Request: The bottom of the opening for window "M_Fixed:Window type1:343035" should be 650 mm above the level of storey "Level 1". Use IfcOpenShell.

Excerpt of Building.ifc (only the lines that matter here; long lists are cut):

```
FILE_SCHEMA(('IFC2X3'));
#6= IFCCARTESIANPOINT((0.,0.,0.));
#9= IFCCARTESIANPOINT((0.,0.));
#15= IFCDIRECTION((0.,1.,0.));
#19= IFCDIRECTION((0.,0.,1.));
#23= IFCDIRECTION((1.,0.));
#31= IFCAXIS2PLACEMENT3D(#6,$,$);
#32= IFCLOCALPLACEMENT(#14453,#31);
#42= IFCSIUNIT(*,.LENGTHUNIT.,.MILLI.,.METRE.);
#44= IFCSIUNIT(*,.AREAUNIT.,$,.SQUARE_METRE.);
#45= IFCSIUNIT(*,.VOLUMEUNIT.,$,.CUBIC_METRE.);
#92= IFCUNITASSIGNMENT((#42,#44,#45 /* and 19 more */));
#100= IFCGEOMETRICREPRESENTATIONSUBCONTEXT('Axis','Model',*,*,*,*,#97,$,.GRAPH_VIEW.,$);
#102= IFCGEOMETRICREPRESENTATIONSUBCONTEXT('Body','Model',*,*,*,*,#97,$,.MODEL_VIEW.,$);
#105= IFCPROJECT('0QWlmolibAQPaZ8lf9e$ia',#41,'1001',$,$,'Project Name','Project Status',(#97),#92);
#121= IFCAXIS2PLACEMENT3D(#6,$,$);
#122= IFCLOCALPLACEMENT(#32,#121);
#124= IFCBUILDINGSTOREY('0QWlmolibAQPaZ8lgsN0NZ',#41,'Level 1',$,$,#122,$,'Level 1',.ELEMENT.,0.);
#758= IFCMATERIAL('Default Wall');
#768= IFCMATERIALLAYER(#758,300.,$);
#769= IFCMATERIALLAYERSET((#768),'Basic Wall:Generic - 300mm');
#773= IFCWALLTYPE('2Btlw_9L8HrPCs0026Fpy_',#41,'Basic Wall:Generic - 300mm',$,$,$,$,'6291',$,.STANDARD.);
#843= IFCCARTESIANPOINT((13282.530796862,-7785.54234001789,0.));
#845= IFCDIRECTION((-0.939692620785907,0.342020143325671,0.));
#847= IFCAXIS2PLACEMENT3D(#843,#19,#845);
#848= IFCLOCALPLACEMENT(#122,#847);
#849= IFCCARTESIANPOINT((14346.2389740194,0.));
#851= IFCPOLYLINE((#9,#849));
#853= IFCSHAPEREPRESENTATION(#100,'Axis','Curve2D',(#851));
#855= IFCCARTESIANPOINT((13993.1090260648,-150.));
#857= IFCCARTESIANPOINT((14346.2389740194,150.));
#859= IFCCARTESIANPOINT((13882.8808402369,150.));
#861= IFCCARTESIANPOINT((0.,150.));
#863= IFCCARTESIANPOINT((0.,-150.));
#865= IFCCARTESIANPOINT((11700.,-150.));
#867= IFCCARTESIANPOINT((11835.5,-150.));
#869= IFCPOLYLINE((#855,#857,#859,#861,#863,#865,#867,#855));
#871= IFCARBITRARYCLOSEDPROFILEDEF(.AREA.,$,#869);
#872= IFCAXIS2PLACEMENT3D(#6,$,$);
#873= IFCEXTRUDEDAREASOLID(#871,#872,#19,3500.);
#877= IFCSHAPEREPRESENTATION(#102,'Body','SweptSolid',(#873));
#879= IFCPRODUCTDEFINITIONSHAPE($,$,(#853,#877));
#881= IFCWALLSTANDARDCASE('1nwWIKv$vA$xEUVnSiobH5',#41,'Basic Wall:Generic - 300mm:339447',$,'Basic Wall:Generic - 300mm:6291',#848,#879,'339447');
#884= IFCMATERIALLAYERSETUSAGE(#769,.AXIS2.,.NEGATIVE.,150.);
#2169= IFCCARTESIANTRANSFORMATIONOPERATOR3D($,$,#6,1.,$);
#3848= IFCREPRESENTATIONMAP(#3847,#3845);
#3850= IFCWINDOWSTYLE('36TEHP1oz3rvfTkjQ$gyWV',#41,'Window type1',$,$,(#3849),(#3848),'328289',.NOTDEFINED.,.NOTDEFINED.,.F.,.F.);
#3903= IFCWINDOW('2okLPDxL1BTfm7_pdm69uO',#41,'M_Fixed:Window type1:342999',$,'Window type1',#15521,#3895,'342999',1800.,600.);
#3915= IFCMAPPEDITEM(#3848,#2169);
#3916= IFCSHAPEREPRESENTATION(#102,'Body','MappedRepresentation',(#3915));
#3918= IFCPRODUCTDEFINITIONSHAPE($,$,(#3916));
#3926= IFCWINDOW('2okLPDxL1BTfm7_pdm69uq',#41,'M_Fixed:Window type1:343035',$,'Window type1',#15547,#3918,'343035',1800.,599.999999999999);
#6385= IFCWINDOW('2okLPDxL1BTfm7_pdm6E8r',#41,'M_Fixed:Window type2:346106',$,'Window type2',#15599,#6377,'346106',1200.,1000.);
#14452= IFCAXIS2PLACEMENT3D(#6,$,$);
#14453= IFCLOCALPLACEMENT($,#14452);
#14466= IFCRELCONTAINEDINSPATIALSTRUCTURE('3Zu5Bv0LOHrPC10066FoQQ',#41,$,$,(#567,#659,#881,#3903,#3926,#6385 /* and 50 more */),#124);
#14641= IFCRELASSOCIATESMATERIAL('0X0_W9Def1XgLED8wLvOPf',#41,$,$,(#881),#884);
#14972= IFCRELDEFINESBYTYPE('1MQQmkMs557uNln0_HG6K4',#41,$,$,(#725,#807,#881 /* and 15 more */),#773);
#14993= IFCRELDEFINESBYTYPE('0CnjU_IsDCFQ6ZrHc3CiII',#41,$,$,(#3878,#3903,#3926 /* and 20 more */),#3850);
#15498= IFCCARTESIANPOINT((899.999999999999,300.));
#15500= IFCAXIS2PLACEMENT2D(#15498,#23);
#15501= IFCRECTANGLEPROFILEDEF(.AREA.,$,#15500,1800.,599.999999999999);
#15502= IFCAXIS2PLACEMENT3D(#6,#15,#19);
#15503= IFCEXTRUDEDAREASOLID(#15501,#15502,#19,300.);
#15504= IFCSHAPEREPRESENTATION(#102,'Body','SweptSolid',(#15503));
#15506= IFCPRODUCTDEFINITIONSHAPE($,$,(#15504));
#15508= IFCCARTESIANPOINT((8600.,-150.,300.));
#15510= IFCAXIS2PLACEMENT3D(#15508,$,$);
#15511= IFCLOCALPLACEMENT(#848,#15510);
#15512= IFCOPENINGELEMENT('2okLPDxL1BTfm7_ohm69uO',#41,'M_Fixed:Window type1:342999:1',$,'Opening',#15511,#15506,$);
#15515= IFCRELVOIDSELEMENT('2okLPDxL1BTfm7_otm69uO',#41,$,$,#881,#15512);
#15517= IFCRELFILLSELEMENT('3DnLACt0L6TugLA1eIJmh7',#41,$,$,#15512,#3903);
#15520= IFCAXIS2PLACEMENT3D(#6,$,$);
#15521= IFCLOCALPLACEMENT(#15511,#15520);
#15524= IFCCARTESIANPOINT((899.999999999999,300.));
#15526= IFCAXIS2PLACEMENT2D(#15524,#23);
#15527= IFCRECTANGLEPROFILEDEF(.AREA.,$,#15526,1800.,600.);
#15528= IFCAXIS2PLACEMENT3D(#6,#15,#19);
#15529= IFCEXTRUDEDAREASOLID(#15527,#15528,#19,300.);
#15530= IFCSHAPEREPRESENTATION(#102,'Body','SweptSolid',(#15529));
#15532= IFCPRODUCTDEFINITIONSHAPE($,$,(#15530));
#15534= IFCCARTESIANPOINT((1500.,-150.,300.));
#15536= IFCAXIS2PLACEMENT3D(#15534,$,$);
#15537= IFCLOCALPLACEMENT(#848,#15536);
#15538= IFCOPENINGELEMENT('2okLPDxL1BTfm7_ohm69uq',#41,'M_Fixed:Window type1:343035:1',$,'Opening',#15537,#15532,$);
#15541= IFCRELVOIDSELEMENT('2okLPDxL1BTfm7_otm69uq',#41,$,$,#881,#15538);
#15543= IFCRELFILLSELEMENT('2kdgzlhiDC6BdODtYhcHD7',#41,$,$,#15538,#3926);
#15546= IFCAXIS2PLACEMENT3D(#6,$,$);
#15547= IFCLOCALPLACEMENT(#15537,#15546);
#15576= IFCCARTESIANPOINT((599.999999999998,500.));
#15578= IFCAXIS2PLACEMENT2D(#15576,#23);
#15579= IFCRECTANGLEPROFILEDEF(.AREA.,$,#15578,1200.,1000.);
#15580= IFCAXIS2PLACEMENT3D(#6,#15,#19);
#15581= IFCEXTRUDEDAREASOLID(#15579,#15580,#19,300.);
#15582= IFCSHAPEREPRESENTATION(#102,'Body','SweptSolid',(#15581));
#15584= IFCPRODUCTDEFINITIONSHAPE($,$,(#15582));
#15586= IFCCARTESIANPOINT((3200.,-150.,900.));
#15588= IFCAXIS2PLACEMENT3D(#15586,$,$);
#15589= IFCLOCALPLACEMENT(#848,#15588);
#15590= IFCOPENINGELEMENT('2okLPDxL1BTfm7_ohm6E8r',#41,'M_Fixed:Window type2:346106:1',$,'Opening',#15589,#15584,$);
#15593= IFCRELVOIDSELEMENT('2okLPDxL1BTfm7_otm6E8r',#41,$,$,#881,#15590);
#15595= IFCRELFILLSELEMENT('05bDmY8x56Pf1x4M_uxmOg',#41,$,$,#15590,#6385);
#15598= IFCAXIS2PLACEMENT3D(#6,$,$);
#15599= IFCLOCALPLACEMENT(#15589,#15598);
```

```python
import numpy as np
import ifcopenshell
import ifcopenshell.api.geometry
import ifcopenshell.geom
import ifcopenshell.util.element
import ifcopenshell.util.placement
import ifcopenshell.util.shape
import ifcopenshell.util.unit

model = ifcopenshell.open("Building.ifc")
unit_scale = ifcopenshell.util.unit.calculate_unit_scale(model)

window = model.by_guid("2okLPDxL1BTfm7_pdm69uq")
opening = window.FillsVoids[0].RelatingOpeningElement
storey = ifcopenshell.util.element.get_container(window, ifc_class="IfcBuildingStorey")
level = ifcopenshell.util.placement.get_local_placement(storey.ObjectPlacement)[2, 3]

# The opening's origin need not be at the sill, so measure its lowest point.
shape = ifcopenshell.geom.create_shape(ifcopenshell.geom.settings(), opening)
bottom = ifcopenshell.util.shape.get_shape_bottom_elevation(shape, shape.geometry) / unit_scale
dz = level + 0.65 / unit_scale - bottom

shift = np.array([0.0, 0.0, dz])
# The window is placed relative to its opening, so it follows when the opening moves.
matrix = ifcopenshell.util.placement.get_local_placement(opening.ObjectPlacement)
matrix[:3, 3] += shift
ifcopenshell.api.geometry.edit_object_placement(
    model, product=opening, matrix=matrix, is_si=False, should_transform_children=True
)

print(f"moved by {dz * unit_scale:+.3f} m")

model.write("Building_edited.ifc")
```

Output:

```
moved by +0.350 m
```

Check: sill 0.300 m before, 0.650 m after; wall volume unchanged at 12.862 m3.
